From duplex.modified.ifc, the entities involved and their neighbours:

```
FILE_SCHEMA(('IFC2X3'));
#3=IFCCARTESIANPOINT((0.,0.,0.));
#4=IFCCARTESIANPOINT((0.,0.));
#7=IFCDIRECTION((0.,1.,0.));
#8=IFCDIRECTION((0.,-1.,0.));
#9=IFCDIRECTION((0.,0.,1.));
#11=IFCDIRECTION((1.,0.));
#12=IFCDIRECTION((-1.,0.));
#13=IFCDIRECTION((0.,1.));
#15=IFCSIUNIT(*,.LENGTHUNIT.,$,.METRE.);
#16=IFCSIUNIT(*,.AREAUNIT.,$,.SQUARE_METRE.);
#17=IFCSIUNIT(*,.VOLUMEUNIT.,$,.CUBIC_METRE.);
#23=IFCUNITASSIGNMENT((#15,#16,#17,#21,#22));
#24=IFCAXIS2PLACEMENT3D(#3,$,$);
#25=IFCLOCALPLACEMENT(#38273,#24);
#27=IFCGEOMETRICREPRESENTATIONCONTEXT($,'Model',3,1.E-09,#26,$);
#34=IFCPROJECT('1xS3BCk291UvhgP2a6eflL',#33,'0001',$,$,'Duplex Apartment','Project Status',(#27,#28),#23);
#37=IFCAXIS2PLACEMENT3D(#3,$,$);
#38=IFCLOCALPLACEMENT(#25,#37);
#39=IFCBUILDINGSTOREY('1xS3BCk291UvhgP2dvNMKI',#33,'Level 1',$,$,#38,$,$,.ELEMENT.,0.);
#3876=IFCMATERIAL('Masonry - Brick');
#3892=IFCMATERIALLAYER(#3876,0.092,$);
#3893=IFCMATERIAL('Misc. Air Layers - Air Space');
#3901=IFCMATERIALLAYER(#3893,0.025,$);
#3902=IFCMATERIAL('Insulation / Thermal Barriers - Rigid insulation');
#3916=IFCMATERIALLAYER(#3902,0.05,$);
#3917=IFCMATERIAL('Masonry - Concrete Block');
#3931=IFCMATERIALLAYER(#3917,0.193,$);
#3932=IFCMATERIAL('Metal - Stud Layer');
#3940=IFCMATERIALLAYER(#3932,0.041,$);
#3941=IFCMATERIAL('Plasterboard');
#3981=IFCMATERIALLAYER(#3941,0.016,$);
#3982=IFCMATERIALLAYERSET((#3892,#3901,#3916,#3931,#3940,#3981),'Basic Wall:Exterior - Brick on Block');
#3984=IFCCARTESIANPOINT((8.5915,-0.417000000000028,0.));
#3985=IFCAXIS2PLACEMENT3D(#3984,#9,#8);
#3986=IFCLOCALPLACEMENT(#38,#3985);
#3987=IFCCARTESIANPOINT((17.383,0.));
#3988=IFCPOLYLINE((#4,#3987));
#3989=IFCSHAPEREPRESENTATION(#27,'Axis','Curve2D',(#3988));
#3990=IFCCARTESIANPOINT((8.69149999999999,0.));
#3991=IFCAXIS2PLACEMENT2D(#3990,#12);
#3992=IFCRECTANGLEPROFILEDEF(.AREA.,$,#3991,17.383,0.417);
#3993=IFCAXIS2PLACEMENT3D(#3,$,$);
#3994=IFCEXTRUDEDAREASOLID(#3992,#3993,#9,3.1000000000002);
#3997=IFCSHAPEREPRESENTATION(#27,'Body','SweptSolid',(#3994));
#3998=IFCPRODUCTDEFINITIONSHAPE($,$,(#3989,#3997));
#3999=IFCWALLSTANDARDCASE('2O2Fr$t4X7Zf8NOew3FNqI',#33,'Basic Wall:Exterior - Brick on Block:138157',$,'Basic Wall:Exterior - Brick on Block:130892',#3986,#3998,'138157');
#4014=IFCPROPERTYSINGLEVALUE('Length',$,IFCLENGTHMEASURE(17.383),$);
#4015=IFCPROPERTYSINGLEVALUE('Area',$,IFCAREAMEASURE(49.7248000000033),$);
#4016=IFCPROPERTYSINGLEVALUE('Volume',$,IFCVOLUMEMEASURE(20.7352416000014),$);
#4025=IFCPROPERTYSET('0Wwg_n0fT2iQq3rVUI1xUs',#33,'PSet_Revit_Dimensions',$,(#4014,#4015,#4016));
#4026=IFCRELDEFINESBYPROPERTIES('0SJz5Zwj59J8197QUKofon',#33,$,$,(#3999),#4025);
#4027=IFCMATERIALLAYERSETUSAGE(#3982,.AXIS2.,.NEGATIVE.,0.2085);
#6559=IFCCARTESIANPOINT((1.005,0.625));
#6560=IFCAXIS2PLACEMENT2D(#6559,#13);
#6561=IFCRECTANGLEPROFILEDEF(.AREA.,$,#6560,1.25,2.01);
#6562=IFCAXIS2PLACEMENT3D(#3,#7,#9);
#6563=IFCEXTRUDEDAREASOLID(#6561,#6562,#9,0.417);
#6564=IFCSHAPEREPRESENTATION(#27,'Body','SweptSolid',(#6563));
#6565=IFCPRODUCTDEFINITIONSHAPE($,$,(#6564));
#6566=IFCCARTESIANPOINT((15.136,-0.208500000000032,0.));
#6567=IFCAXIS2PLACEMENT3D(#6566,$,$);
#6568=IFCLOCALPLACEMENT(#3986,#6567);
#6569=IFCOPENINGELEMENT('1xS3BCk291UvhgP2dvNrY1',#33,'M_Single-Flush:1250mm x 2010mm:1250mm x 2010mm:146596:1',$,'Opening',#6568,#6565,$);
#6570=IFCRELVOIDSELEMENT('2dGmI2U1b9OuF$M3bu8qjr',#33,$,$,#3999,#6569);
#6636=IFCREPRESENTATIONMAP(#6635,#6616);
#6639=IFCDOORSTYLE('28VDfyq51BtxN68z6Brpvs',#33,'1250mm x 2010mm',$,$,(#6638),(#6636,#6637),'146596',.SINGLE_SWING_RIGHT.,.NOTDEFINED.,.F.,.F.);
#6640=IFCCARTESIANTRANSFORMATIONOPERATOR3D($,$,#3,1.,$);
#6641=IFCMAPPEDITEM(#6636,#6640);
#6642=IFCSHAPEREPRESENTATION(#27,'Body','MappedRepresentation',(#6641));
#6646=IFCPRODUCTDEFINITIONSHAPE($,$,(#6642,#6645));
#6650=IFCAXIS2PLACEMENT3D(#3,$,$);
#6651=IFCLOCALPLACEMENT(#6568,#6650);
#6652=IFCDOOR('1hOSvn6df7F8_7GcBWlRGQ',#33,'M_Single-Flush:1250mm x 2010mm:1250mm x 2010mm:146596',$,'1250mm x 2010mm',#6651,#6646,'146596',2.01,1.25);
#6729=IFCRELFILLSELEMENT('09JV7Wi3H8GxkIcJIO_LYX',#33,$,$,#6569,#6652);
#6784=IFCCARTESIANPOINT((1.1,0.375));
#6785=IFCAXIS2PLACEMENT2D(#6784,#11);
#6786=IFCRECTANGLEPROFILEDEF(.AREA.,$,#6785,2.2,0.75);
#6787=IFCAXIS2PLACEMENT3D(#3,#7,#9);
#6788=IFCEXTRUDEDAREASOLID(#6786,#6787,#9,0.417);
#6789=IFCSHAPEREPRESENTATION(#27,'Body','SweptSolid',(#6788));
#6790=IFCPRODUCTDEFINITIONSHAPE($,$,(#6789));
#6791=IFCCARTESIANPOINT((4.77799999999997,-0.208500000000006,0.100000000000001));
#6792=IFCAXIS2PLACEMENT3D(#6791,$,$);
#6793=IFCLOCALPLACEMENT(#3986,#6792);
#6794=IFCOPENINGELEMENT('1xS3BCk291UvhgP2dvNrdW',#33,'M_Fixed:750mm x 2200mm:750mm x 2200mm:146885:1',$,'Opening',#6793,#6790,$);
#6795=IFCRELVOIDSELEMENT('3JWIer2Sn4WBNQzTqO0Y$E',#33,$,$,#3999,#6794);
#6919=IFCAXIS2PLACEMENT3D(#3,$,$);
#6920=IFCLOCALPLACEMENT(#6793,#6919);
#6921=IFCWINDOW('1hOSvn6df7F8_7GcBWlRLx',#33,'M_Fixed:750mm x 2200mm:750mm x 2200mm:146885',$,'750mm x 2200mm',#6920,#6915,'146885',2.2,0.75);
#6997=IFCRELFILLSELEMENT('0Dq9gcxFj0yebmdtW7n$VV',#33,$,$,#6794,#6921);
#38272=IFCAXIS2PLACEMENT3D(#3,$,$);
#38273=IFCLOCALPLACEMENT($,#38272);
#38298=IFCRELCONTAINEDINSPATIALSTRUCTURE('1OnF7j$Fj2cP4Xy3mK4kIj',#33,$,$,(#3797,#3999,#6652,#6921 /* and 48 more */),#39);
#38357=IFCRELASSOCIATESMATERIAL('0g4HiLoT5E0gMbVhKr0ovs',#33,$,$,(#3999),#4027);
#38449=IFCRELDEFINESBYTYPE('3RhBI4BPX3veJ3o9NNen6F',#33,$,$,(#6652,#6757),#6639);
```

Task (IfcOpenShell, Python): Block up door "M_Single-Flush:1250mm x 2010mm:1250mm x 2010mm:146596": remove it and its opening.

```python
import ifcopenshell
import ifcopenshell.api.feature
import ifcopenshell.api.pset
import ifcopenshell.api.root
import ifcopenshell.geom
import ifcopenshell.util.element
import ifcopenshell.util.shape
import ifcopenshell.util.unit

model = ifcopenshell.open("duplex.modified.ifc")
area_scale = ifcopenshell.util.unit.calculate_unit_scale(model, "AREAUNIT")
volume_scale = ifcopenshell.util.unit.calculate_unit_scale(model, "VOLUMEUNIT")
settings = ifcopenshell.geom.settings()


def volume(element):
    """Net volume in cubic metres, openings subtracted."""
    shape = ifcopenshell.geom.create_shape(settings, element)
    return ifcopenshell.util.shape.get_volume(shape.geometry)


door = model.by_guid("1hOSvn6df7F8_7GcBWlRGQ")
opening = door.FillsVoids[0].RelatingOpeningElement
wall = opening.VoidsElements[0].RelatingBuildingElement
before = volume(wall)

ifcopenshell.api.root.remove_product(model, product=door)
ifcopenshell.api.feature.remove_feature(model, feature=opening)

after = volume(wall)
thickness = 0.417  # wall thickness in metres

# Update the wall's stored quantities.
pset = model.by_id(ifcopenshell.util.element.get_pset(wall, "PSet_Revit_Dimensions", should_inherit=False)["id"])
ifcopenshell.api.pset.edit_pset(model, pset=pset, properties={
    "Area": model.create_entity("IfcAreaMeasure", after / thickness / area_scale),
    "Volume": model.create_entity("IfcVolumeMeasure", after / volume_scale),
})

print(f"wall volume {before:.3f} -> {after:.3f} m3")

model.write("duplex.modified_v2.ifc")
```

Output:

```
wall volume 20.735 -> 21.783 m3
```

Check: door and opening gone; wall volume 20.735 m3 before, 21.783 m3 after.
